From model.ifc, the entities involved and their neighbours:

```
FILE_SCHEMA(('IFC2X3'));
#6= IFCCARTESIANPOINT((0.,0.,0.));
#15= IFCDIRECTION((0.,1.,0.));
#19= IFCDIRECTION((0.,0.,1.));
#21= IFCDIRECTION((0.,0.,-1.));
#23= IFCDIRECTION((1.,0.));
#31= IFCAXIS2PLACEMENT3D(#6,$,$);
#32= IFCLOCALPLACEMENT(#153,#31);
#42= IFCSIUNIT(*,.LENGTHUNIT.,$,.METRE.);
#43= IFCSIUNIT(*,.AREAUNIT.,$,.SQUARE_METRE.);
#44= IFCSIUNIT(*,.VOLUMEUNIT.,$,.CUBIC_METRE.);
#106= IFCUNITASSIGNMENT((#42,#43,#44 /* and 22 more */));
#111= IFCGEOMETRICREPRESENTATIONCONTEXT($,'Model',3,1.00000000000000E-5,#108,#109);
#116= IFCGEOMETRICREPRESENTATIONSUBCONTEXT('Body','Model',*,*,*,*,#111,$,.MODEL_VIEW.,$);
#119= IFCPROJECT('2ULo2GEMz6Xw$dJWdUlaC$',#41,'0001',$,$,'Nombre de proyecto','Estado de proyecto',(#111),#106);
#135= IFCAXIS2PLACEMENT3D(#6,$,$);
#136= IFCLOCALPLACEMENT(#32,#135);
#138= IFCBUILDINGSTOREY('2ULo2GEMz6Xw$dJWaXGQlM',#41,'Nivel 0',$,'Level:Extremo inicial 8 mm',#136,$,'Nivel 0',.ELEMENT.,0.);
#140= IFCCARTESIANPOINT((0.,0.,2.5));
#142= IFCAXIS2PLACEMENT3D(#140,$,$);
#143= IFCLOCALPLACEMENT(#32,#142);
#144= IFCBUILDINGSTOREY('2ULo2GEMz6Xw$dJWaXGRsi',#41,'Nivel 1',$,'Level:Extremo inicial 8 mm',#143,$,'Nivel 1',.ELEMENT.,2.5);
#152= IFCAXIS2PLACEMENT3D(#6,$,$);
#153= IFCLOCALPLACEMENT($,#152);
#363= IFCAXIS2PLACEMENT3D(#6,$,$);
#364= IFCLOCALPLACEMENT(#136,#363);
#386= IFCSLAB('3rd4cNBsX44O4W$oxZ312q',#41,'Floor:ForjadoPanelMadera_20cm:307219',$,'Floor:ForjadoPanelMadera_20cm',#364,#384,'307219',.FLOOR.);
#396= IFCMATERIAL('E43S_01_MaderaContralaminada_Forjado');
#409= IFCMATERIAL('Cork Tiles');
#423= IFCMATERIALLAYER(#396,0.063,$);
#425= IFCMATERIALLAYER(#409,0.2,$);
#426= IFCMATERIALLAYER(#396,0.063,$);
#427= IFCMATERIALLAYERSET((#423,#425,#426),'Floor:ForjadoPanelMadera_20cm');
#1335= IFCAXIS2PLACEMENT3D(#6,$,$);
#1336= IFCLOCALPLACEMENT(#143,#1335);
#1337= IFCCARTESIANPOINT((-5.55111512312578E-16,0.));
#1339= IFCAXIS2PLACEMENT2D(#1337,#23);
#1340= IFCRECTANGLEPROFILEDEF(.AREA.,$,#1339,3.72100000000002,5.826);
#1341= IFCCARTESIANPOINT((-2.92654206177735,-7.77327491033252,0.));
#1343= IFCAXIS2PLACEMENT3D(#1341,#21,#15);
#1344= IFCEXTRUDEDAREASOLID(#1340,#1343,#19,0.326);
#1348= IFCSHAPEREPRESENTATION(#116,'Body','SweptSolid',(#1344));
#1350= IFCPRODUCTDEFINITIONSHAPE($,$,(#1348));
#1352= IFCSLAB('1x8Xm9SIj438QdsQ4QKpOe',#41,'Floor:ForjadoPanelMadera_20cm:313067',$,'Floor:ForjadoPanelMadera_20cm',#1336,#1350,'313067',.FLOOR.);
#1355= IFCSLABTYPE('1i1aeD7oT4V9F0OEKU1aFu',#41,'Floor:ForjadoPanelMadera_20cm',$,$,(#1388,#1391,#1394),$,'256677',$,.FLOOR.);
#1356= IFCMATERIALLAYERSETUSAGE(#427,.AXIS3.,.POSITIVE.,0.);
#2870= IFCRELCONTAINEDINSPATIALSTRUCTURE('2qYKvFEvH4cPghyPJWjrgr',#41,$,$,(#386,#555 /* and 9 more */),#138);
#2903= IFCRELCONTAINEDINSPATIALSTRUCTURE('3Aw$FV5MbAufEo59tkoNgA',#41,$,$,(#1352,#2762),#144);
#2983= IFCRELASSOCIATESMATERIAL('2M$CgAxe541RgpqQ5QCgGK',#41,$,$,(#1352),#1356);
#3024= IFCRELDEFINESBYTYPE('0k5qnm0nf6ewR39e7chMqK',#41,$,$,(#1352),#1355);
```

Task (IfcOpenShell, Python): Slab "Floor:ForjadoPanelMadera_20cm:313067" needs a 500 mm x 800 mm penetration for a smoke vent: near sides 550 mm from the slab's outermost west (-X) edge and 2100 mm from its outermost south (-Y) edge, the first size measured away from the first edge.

```python
import numpy as np
import ifcopenshell
import ifcopenshell.api.feature
import ifcopenshell.api.geometry
import ifcopenshell.api.root
import ifcopenshell.geom
import ifcopenshell.util.placement
import ifcopenshell.util.representation
import ifcopenshell.util.shape
import ifcopenshell.util.unit

model = ifcopenshell.open("model.ifc")
unit_scale = ifcopenshell.util.unit.calculate_unit_scale(model)
settings = ifcopenshell.geom.settings()


def volume(element):
    """Net volume in cubic metres, openings subtracted."""
    shape = ifcopenshell.geom.create_shape(settings, element)
    return ifcopenshell.util.shape.get_volume(shape.geometry)


slab = model.by_guid("1x8Xm9SIj438QdsQ4QKpOe")
before = volume(slab)

# Extent in the slab's own axes, in metres. The edges named are its -X and -Y sides.
slab_shape = ifcopenshell.geom.create_shape(settings, slab)
vertices = ifcopenshell.util.shape.get_vertices(slab_shape.geometry)
x_min, y_min, bottom = vertices.min(axis=0)
top = vertices[:, 2].max()

opening = ifcopenshell.api.root.create_entity(model, ifc_class="IfcOpeningElement", name="Smoke vent opening")
context = ifcopenshell.util.representation.get_context(model, "Model", "Body", "MODEL_VIEW")
width, depth = 0.5, 0.8
outline = [(0.0, 0.0), (width, 0.0), (width, depth), (0.0, depth), (0.0, 0.0)]
# Overshoot both faces by 50 mm so the cut is clean.
shape = ifcopenshell.api.geometry.add_slab_representation(
    model, context=context, depth=top - bottom + 0.1, polyline=outline
)
ifcopenshell.api.geometry.assign_representation(model, product=opening, representation=shape)

matrix = ifcopenshell.util.placement.get_local_placement(slab.ObjectPlacement)
matrix[:, 3] = matrix @ np.append(np.array([x_min + 0.55, y_min + 2.1, bottom - 0.05]) / unit_scale, 1.0)
ifcopenshell.api.geometry.edit_object_placement(model, product=opening, matrix=matrix, is_si=False)
ifcopenshell.api.feature.add_feature(model, feature=opening, element=slab)

after = volume(slab)

print(f"slab volume {before:.3f} -> {after:.3f} m3")

model.write("model_edited.ifc")
```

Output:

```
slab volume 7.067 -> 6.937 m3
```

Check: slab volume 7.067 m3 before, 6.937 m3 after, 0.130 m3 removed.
